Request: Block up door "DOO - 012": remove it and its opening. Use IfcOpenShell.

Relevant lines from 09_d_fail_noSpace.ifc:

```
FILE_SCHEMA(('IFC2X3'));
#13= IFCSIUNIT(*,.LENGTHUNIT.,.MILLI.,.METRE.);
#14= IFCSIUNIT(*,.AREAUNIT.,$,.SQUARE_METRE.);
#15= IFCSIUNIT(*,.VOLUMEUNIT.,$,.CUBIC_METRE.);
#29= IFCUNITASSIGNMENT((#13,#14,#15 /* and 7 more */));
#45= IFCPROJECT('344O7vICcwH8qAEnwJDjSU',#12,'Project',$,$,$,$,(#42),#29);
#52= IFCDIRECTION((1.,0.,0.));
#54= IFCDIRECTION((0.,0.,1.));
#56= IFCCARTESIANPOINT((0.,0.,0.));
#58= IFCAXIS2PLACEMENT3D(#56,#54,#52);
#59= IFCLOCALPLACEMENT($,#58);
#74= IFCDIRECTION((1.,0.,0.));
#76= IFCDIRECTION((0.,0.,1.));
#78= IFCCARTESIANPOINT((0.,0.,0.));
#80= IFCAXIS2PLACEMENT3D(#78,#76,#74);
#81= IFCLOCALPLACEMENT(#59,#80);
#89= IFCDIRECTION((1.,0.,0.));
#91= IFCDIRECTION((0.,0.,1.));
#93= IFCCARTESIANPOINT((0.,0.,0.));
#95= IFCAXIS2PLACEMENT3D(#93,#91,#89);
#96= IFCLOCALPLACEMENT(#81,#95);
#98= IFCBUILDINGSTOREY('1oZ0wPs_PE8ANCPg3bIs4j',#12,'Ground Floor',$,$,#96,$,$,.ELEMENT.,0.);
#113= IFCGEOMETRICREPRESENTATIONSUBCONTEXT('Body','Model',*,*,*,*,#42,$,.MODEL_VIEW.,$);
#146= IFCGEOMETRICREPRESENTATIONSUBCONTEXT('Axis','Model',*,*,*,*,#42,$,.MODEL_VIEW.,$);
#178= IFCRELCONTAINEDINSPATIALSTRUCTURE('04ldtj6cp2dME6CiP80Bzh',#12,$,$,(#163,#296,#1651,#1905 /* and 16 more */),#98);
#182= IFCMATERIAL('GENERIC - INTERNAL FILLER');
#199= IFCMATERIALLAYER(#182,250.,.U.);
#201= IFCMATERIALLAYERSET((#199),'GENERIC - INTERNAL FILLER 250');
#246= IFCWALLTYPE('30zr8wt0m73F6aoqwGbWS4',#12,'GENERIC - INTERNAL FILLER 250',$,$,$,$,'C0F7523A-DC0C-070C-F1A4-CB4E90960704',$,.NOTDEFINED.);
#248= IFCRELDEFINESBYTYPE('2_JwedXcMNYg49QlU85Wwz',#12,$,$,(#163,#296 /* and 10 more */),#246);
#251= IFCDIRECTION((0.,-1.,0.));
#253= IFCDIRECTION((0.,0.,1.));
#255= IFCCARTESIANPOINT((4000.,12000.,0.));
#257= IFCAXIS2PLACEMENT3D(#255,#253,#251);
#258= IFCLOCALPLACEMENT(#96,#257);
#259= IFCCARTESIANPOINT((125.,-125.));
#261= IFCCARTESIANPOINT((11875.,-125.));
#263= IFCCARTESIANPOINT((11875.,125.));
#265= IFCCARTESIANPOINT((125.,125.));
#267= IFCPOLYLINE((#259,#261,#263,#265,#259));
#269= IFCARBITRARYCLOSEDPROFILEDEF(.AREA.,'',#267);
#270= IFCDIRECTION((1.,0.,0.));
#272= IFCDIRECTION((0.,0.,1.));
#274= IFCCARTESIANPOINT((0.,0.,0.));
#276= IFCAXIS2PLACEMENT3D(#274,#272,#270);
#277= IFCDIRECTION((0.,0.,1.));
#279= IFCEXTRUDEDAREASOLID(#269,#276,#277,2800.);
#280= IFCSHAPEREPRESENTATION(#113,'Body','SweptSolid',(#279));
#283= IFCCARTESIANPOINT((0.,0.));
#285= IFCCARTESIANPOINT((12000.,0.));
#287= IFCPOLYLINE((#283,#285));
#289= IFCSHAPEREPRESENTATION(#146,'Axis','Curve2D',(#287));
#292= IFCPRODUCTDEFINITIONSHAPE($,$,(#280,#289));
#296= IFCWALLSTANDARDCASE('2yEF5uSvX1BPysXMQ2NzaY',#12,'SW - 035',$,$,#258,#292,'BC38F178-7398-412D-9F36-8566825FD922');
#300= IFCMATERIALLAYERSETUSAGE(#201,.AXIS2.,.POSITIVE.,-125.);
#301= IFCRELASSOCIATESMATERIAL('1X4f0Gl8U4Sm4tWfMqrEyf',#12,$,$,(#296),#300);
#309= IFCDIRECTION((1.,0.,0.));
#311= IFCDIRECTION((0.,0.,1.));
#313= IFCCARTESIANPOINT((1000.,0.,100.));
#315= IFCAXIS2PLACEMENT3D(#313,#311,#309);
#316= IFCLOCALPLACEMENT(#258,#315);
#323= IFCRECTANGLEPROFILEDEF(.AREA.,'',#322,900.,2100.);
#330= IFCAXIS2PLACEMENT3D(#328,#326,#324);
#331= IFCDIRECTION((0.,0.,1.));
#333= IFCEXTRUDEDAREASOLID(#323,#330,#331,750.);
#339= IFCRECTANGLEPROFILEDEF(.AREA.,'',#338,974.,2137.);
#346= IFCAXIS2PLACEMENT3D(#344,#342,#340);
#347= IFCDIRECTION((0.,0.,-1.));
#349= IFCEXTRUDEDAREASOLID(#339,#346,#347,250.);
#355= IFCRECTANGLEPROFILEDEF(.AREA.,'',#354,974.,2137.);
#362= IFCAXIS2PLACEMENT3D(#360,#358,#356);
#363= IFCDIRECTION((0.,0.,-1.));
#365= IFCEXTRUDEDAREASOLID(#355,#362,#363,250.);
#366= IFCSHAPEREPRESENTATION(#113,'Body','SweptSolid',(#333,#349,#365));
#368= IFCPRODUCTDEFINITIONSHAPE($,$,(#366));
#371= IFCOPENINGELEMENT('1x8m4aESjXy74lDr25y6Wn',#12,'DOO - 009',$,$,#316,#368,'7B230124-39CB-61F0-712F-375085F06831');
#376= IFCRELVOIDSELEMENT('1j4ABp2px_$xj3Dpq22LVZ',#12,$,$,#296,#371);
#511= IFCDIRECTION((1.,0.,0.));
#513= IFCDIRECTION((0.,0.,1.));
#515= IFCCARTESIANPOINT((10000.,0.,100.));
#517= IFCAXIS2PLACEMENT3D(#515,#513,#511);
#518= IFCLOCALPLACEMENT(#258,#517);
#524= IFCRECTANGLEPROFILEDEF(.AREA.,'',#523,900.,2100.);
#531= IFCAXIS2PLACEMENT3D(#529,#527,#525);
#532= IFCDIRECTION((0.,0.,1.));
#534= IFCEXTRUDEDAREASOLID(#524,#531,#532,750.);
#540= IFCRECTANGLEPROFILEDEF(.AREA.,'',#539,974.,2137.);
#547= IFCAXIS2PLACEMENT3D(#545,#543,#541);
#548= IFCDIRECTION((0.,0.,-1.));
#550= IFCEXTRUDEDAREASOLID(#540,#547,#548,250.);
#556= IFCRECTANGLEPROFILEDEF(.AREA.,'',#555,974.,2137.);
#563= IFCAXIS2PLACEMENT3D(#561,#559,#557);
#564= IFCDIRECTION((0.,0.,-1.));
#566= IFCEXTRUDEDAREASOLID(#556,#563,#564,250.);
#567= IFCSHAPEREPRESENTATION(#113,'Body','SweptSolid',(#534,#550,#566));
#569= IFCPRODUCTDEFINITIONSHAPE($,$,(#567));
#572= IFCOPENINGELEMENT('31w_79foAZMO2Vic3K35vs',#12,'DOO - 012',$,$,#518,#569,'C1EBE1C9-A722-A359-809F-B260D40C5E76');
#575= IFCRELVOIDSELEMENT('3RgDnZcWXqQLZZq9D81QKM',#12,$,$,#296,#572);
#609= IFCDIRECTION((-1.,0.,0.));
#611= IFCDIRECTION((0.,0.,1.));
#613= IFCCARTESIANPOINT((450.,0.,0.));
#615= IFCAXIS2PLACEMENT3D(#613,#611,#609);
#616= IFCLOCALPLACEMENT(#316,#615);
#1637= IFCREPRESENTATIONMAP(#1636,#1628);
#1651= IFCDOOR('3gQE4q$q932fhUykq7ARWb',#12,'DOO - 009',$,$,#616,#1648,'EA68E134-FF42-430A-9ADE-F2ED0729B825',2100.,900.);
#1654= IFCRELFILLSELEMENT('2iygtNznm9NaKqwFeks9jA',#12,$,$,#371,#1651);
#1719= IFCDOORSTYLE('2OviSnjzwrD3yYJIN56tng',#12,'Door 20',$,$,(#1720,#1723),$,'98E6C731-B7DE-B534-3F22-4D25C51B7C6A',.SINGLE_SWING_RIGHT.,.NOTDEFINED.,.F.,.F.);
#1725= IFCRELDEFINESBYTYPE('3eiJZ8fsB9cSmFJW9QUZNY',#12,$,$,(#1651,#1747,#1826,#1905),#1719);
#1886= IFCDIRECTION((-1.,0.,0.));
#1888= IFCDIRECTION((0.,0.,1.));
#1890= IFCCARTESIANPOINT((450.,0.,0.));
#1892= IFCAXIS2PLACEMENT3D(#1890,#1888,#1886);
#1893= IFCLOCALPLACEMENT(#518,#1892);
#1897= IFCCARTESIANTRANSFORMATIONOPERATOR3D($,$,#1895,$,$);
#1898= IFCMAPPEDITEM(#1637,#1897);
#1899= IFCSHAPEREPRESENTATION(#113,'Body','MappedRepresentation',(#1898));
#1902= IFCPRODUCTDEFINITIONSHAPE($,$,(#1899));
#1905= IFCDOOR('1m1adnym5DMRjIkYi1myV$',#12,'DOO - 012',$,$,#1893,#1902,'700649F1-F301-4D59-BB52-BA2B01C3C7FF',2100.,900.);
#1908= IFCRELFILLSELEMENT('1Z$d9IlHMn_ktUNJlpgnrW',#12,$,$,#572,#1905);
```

```python
import ifcopenshell
import ifcopenshell.api.feature
import ifcopenshell.api.root
import ifcopenshell.geom
import ifcopenshell.util.shape

model = ifcopenshell.open("09_d_fail_noSpace.ifc")
settings = ifcopenshell.geom.settings()


def volume(element):
    """Net volume in cubic metres, openings subtracted."""
    shape = ifcopenshell.geom.create_shape(settings, element)
    return ifcopenshell.util.shape.get_volume(shape.geometry)


door = model.by_id(1905)
opening = door.FillsVoids[0].RelatingOpeningElement
wall = opening.VoidsElements[0].RelatingBuildingElement
before = volume(wall)

ifcopenshell.api.root.remove_product(model, product=door)
ifcopenshell.api.feature.remove_feature(model, feature=opening)

after = volume(wall)

print(f"wall volume {before:.3f} -> {after:.3f} m3")

model.write("09_d_fail_noSpace_rev.ifc")
```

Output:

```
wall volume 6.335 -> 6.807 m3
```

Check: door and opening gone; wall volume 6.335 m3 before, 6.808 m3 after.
